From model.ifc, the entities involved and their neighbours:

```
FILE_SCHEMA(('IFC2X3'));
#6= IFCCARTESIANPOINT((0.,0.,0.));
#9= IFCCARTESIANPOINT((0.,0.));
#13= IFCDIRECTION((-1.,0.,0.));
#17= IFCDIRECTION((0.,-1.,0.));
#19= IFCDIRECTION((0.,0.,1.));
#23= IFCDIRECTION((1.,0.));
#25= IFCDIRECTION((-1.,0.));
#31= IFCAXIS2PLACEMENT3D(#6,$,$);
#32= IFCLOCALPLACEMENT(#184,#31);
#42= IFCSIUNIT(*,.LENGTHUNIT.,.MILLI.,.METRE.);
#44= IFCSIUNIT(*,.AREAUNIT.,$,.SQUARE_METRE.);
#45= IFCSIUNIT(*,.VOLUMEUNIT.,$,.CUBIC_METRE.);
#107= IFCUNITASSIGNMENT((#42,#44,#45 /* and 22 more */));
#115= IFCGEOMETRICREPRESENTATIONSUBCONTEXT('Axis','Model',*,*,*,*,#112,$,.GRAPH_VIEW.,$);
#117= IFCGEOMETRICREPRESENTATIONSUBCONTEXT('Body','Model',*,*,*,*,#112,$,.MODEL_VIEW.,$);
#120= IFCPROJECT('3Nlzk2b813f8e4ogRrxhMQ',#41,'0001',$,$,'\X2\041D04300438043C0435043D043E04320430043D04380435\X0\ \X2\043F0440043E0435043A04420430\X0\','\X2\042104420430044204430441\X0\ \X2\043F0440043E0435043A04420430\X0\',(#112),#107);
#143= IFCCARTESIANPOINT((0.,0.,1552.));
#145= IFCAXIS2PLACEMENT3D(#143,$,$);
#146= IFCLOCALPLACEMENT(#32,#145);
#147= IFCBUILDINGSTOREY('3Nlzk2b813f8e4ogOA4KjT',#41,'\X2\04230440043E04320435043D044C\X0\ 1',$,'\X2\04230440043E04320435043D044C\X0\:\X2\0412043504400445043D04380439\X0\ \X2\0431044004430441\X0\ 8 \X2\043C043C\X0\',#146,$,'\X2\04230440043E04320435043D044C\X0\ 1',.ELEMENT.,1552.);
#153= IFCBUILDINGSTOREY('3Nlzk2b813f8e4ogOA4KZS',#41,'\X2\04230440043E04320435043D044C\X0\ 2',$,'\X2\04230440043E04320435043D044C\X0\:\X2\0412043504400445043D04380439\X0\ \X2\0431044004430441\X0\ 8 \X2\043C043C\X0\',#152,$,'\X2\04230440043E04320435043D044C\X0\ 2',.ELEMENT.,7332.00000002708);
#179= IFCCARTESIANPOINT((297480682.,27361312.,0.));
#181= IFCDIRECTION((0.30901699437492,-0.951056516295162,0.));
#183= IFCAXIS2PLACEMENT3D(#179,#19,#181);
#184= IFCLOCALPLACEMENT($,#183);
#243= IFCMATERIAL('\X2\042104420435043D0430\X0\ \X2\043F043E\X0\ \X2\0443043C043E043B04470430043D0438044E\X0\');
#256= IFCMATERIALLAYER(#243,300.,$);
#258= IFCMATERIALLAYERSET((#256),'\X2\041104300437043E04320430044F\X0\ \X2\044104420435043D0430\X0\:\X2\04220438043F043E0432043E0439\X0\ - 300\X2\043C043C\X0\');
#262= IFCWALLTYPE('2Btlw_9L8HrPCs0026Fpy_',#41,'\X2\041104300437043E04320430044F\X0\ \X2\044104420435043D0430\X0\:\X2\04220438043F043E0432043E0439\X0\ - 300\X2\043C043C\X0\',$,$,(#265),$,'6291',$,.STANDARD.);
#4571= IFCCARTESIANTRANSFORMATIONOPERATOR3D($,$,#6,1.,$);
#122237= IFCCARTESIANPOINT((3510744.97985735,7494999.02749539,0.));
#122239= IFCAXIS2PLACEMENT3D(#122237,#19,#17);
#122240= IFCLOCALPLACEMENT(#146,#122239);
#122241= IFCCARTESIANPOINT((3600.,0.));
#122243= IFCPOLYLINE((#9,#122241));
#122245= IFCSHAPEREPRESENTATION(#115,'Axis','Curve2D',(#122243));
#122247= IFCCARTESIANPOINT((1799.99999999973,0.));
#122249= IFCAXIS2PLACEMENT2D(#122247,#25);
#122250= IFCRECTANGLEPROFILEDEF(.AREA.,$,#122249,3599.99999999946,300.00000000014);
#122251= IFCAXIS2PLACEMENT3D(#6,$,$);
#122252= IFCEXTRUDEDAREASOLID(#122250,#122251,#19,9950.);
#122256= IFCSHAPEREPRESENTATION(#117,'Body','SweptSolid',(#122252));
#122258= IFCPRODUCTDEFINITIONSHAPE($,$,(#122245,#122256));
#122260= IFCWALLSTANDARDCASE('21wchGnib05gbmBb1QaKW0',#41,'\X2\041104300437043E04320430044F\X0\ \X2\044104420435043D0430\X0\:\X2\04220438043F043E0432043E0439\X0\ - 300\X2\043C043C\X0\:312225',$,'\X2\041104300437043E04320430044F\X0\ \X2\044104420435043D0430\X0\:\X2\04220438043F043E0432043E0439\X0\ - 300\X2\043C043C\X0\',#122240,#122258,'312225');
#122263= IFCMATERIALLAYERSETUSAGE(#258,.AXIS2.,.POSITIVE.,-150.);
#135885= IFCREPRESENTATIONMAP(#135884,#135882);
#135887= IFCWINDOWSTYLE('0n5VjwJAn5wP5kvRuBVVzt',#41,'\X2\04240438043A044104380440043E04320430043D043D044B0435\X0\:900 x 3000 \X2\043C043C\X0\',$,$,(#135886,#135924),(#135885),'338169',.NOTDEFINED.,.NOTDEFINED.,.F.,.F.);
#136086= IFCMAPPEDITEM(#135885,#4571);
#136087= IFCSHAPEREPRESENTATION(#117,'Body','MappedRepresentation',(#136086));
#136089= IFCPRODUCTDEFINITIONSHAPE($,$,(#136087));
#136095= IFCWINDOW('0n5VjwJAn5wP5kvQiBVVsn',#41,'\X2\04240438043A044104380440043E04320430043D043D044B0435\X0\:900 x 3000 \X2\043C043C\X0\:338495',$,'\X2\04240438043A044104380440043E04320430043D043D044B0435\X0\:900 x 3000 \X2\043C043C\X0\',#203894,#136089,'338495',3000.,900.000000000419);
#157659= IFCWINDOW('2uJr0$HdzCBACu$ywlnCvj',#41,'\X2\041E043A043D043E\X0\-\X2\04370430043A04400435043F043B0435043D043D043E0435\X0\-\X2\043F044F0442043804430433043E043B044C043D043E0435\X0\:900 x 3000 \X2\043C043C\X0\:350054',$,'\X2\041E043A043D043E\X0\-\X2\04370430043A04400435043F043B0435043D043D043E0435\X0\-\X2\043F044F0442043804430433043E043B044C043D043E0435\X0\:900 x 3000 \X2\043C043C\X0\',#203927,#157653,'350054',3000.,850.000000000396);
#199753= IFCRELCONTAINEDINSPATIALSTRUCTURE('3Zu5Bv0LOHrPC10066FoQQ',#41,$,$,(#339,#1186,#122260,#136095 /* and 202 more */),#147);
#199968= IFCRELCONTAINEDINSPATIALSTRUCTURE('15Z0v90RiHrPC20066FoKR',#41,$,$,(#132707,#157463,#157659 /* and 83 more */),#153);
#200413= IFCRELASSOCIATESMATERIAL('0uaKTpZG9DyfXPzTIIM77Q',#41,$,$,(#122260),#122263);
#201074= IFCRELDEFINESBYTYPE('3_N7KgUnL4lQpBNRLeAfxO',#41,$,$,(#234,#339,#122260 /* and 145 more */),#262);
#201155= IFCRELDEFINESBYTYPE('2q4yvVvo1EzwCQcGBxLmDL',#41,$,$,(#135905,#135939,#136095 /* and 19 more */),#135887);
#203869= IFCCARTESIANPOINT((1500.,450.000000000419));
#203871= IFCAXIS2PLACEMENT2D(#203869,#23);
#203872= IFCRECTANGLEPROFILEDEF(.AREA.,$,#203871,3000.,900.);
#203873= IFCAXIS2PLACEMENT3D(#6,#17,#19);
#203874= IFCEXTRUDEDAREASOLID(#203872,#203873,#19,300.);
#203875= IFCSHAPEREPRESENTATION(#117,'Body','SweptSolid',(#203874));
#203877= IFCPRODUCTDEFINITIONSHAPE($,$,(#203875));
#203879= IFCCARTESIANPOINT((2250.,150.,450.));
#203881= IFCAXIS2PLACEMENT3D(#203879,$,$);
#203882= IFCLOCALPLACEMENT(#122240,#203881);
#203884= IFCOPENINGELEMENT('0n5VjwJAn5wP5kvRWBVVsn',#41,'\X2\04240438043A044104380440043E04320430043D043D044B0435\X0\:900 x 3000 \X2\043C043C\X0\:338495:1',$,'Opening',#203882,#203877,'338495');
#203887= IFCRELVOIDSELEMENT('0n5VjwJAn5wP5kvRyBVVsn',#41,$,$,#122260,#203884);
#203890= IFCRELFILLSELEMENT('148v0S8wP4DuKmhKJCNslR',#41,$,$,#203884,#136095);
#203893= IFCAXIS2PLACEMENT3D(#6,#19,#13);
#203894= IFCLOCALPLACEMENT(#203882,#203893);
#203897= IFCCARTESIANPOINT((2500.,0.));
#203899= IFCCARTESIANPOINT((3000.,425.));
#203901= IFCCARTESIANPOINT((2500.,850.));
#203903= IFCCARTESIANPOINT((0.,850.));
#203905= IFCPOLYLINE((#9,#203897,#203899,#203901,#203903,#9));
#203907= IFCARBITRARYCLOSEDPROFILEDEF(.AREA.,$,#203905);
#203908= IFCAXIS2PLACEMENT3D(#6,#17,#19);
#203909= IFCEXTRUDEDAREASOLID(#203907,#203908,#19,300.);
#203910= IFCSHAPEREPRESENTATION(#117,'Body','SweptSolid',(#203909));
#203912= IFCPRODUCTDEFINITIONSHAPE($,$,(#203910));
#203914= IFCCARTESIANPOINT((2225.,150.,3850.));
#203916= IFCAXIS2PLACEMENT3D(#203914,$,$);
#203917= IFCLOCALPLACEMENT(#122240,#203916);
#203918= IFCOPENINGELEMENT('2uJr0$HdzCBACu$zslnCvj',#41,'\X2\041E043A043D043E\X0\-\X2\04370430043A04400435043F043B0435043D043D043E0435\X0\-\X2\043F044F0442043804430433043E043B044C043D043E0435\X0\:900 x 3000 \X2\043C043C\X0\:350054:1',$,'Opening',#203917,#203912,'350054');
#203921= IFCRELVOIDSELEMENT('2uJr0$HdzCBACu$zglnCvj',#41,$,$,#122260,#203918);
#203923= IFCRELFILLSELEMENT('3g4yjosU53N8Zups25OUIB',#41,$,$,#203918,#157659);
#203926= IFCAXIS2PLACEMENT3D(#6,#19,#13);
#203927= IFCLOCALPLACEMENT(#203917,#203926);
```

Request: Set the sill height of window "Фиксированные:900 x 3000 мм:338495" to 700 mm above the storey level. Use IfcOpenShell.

```python
import numpy as np
import ifcopenshell
import ifcopenshell.api.geometry
import ifcopenshell.geom
import ifcopenshell.util.element
import ifcopenshell.util.placement
import ifcopenshell.util.shape
import ifcopenshell.util.unit

model = ifcopenshell.open("model.ifc")
unit_scale = ifcopenshell.util.unit.calculate_unit_scale(model)

window = model.by_guid("0n5VjwJAn5wP5kvQiBVVsn")
opening = window.FillsVoids[0].RelatingOpeningElement
storey = ifcopenshell.util.element.get_container(window, ifc_class="IfcBuildingStorey")
level = ifcopenshell.util.placement.get_local_placement(storey.ObjectPlacement)[2, 3]

# The opening's origin need not be at the sill, so measure its lowest point.
shape = ifcopenshell.geom.create_shape(ifcopenshell.geom.settings(), opening)
bottom = ifcopenshell.util.shape.get_shape_bottom_elevation(shape, shape.geometry) / unit_scale
dz = level + 700.0 - bottom

shift = np.array([0.0, 0.0, dz])
# The window is placed relative to its opening, so it follows when the opening moves.
matrix = ifcopenshell.util.placement.get_local_placement(opening.ObjectPlacement)
matrix[:3, 3] += shift
ifcopenshell.api.geometry.edit_object_placement(
    model, product=opening, matrix=matrix, is_si=False, should_transform_children=True
)

print(f"moved by {dz * unit_scale:+.3f} m")

model.write("model-out.ifc")
```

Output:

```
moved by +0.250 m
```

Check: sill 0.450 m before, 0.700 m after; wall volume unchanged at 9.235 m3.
